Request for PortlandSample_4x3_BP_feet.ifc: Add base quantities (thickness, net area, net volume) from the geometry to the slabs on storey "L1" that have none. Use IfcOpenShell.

First a look at what the model holds.

```python
import ifcopenshell
import ifcopenshell.util.element
import ifcopenshell.util.unit

model = ifcopenshell.open("PortlandSample_4x3_BP_feet.ifc")
print(model.schema)
for unit_type in ("LENGTHUNIT", "AREAUNIT", "VOLUMEUNIT"):
    print(unit_type, ifcopenshell.util.unit.calculate_unit_scale(model, unit_type))
storey = next(s for s in model.by_type("IfcBuildingStorey") if s.Name == "L1")
slabs = [e for e in ifcopenshell.util.element.get_decomposition(storey) if e.is_a("IfcSlab")]
for e in sorted(slabs, key=lambda e: e.id()):
    print(e.id(), e.is_a(), e.Name, list(ifcopenshell.util.element.get_psets(e, qtos_only=True)), sep=" | ")
```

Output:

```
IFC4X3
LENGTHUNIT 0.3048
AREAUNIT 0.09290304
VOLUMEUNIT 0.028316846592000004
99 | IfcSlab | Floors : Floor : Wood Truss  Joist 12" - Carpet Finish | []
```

```python
import ifcopenshell
import ifcopenshell.api.pset
import ifcopenshell.geom
import ifcopenshell.util.element
import ifcopenshell.util.shape
import ifcopenshell.util.unit

model = ifcopenshell.open("PortlandSample_4x3_BP_feet.ifc")
unit_scale = ifcopenshell.util.unit.calculate_unit_scale(model)
area_scale = ifcopenshell.util.unit.calculate_unit_scale(model, "AREAUNIT")
volume_scale = ifcopenshell.util.unit.calculate_unit_scale(model, "VOLUMEUNIT")
settings = ifcopenshell.geom.settings()

storey = next(s for s in model.by_type("IfcBuildingStorey") if s.Name == "L1")
slabs = [e for e in ifcopenshell.util.element.get_decomposition(storey) if e.is_a("IfcSlab")]

for e in sorted(slabs, key=lambda e: e.id()):
    if ifcopenshell.util.element.get_psets(e, qtos_only=True, should_inherit=False):
        continue
    # Geometry comes back in metres, in the element's own axes.
    shape = ifcopenshell.geom.create_shape(settings, e)
    values = {
        "Width": ifcopenshell.util.shape.get_z(shape.geometry) / unit_scale,
        "NetArea": ifcopenshell.util.shape.get_footprint_area(shape.geometry) / area_scale,
        "NetVolume": ifcopenshell.util.shape.get_volume(shape.geometry) / volume_scale,
    }
    qto = ifcopenshell.api.pset.add_qto(model, product=e, name="Qto_SlabBaseQuantities")
    ifcopenshell.api.pset.edit_qto(model, qto=qto, properties=values)
    print(e.id(), {k: round(v, 3) for k, v in values.items()})

model.write("PortlandSample_4x3_BP_feet_updated.ifc")
```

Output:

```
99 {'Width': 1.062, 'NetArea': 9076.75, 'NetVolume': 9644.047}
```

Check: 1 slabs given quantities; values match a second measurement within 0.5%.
